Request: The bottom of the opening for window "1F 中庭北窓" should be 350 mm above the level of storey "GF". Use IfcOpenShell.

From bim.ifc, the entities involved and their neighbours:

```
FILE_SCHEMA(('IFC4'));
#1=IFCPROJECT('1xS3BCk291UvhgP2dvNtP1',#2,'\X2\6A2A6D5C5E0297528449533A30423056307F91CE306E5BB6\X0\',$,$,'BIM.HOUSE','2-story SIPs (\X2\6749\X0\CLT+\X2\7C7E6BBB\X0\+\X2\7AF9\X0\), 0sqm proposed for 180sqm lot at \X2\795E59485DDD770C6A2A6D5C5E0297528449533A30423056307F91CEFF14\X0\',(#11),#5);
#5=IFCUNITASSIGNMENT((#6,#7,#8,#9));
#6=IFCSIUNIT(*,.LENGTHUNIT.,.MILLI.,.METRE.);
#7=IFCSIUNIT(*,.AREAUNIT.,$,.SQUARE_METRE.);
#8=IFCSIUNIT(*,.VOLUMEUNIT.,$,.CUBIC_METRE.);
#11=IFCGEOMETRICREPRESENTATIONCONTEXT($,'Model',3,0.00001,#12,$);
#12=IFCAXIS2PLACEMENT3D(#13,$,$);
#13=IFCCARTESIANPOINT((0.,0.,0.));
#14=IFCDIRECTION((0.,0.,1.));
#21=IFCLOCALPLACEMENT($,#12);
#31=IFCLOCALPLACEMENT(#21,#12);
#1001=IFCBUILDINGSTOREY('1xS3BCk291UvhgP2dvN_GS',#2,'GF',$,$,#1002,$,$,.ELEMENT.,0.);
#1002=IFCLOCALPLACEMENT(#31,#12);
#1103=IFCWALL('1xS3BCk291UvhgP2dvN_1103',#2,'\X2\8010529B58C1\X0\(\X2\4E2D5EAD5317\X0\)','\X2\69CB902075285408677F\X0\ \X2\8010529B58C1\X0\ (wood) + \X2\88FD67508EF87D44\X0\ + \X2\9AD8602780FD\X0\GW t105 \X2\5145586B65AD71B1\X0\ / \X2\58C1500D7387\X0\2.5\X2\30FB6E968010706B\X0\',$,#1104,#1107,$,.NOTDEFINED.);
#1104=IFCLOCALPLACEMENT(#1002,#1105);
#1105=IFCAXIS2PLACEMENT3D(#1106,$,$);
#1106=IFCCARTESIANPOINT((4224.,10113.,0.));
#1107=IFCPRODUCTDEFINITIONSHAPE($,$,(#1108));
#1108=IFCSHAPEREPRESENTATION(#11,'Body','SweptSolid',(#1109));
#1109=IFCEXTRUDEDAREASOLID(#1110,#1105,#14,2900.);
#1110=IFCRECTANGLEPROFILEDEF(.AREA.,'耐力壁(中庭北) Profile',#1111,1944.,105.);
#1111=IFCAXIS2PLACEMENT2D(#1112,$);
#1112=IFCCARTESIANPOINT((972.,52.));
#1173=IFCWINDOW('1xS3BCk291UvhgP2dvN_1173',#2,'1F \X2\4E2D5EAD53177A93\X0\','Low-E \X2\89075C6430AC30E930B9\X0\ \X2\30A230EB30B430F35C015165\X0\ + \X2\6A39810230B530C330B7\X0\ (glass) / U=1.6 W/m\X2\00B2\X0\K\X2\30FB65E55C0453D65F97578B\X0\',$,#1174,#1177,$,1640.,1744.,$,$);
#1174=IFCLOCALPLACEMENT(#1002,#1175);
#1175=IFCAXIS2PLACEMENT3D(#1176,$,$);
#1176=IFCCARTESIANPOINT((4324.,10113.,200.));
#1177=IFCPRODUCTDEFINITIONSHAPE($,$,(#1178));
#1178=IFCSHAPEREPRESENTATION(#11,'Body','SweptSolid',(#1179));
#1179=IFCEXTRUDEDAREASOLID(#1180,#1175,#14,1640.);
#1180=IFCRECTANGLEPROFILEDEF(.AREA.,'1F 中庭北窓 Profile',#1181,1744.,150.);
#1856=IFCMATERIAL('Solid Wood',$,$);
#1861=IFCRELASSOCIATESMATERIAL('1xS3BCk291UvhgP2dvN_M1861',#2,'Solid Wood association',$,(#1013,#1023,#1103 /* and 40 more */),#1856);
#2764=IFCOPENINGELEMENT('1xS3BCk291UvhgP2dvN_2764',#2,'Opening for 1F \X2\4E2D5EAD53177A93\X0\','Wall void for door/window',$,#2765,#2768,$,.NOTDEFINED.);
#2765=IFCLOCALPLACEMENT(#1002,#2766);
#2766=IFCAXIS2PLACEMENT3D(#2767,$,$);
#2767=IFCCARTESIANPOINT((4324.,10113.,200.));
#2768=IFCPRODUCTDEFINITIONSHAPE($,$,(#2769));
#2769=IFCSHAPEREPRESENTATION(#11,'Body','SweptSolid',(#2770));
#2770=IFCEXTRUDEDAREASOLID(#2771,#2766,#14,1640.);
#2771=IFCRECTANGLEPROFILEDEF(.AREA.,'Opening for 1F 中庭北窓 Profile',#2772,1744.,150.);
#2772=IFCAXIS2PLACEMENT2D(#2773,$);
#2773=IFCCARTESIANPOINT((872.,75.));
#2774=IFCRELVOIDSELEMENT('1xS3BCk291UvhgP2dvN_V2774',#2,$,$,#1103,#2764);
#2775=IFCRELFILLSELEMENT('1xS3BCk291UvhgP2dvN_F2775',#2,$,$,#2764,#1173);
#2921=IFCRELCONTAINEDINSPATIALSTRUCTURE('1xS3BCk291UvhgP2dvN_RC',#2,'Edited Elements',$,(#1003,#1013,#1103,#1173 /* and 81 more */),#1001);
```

```python
import numpy as np
import ifcopenshell
import ifcopenshell.api.geometry
import ifcopenshell.geom
import ifcopenshell.util.element
import ifcopenshell.util.placement
import ifcopenshell.util.shape
import ifcopenshell.util.unit

model = ifcopenshell.open("bim.ifc")
unit_scale = ifcopenshell.util.unit.calculate_unit_scale(model)

window = model.by_guid("1xS3BCk291UvhgP2dvN_1173")
opening = window.FillsVoids[0].RelatingOpeningElement
storey = ifcopenshell.util.element.get_container(window, ifc_class="IfcBuildingStorey")
level = ifcopenshell.util.placement.get_local_placement(storey.ObjectPlacement)[2, 3]

# The opening's origin need not be at the sill, so measure its lowest point.
shape = ifcopenshell.geom.create_shape(ifcopenshell.geom.settings(), opening)
bottom = ifcopenshell.util.shape.get_shape_bottom_elevation(shape, shape.geometry) / unit_scale
dz = level + 350.0 - bottom

shift = np.array([0.0, 0.0, dz])
# The window is not placed relative to its opening, so move both.
for product in (opening, window):
    matrix = ifcopenshell.util.placement.get_local_placement(product.ObjectPlacement)
    matrix[:3, 3] += shift
    ifcopenshell.api.geometry.edit_object_placement(model, product=product, matrix=matrix, is_si=False)

print(f"moved by {dz * unit_scale:+.3f} m")

model.write("bim-out.ifc")
```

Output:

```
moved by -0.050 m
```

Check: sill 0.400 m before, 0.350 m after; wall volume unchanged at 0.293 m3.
